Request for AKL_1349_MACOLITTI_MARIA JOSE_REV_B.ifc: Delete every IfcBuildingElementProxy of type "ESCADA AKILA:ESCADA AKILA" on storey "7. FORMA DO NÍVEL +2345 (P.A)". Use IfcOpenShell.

First a look at what the model holds.

```python
import ifcopenshell
import ifcopenshell.util.element

model = ifcopenshell.open("AKL_1349_MACOLITTI_MARIA JOSE_REV_B.ifc")
print(model.schema)
storey = next(s for s in model.by_type("IfcBuildingStorey") if s.Name == "7. FORMA DO NÍVEL +2345 (P.A)")
proxies = [e for e in ifcopenshell.util.element.get_decomposition(storey) if e.is_a("IfcBuildingElementProxy")]
seen = {}
for e in proxies:
    element_type = ifcopenshell.util.element.get_type(e)
    name = element_type.Name if element_type not in (None, e) else None
    seen[name] = seen.get(name, 0) + 1
for name, count in sorted(seen.items(), key=str):
    print(count, "x", name)
```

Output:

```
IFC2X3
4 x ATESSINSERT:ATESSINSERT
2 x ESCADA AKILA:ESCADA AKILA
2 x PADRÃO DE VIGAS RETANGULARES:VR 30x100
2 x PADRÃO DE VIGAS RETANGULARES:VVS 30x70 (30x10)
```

```python
import ifcopenshell
import ifcopenshell.api.root
import ifcopenshell.util.element

model = ifcopenshell.open("AKL_1349_MACOLITTI_MARIA JOSE_REV_B.ifc")

storey = next(s for s in model.by_type("IfcBuildingStorey") if s.Name == "7. FORMA DO NÍVEL +2345 (P.A)")
proxies = [e for e in ifcopenshell.util.element.get_decomposition(storey) if e.is_a("IfcBuildingElementProxy")]
targets = [e for e in proxies if (t := ifcopenshell.util.element.get_type(e)) not in (None, e) and t.Name == "ESCADA AKILA:ESCADA AKILA"]

for e in targets:
    ifcopenshell.api.root.remove_product(model, product=e)
print(len(targets), "removed")

model.write("AKL_1349_MACOLITTI_MARIA JOSE_REV_B_v2.ifc")
```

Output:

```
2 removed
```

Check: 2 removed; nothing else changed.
